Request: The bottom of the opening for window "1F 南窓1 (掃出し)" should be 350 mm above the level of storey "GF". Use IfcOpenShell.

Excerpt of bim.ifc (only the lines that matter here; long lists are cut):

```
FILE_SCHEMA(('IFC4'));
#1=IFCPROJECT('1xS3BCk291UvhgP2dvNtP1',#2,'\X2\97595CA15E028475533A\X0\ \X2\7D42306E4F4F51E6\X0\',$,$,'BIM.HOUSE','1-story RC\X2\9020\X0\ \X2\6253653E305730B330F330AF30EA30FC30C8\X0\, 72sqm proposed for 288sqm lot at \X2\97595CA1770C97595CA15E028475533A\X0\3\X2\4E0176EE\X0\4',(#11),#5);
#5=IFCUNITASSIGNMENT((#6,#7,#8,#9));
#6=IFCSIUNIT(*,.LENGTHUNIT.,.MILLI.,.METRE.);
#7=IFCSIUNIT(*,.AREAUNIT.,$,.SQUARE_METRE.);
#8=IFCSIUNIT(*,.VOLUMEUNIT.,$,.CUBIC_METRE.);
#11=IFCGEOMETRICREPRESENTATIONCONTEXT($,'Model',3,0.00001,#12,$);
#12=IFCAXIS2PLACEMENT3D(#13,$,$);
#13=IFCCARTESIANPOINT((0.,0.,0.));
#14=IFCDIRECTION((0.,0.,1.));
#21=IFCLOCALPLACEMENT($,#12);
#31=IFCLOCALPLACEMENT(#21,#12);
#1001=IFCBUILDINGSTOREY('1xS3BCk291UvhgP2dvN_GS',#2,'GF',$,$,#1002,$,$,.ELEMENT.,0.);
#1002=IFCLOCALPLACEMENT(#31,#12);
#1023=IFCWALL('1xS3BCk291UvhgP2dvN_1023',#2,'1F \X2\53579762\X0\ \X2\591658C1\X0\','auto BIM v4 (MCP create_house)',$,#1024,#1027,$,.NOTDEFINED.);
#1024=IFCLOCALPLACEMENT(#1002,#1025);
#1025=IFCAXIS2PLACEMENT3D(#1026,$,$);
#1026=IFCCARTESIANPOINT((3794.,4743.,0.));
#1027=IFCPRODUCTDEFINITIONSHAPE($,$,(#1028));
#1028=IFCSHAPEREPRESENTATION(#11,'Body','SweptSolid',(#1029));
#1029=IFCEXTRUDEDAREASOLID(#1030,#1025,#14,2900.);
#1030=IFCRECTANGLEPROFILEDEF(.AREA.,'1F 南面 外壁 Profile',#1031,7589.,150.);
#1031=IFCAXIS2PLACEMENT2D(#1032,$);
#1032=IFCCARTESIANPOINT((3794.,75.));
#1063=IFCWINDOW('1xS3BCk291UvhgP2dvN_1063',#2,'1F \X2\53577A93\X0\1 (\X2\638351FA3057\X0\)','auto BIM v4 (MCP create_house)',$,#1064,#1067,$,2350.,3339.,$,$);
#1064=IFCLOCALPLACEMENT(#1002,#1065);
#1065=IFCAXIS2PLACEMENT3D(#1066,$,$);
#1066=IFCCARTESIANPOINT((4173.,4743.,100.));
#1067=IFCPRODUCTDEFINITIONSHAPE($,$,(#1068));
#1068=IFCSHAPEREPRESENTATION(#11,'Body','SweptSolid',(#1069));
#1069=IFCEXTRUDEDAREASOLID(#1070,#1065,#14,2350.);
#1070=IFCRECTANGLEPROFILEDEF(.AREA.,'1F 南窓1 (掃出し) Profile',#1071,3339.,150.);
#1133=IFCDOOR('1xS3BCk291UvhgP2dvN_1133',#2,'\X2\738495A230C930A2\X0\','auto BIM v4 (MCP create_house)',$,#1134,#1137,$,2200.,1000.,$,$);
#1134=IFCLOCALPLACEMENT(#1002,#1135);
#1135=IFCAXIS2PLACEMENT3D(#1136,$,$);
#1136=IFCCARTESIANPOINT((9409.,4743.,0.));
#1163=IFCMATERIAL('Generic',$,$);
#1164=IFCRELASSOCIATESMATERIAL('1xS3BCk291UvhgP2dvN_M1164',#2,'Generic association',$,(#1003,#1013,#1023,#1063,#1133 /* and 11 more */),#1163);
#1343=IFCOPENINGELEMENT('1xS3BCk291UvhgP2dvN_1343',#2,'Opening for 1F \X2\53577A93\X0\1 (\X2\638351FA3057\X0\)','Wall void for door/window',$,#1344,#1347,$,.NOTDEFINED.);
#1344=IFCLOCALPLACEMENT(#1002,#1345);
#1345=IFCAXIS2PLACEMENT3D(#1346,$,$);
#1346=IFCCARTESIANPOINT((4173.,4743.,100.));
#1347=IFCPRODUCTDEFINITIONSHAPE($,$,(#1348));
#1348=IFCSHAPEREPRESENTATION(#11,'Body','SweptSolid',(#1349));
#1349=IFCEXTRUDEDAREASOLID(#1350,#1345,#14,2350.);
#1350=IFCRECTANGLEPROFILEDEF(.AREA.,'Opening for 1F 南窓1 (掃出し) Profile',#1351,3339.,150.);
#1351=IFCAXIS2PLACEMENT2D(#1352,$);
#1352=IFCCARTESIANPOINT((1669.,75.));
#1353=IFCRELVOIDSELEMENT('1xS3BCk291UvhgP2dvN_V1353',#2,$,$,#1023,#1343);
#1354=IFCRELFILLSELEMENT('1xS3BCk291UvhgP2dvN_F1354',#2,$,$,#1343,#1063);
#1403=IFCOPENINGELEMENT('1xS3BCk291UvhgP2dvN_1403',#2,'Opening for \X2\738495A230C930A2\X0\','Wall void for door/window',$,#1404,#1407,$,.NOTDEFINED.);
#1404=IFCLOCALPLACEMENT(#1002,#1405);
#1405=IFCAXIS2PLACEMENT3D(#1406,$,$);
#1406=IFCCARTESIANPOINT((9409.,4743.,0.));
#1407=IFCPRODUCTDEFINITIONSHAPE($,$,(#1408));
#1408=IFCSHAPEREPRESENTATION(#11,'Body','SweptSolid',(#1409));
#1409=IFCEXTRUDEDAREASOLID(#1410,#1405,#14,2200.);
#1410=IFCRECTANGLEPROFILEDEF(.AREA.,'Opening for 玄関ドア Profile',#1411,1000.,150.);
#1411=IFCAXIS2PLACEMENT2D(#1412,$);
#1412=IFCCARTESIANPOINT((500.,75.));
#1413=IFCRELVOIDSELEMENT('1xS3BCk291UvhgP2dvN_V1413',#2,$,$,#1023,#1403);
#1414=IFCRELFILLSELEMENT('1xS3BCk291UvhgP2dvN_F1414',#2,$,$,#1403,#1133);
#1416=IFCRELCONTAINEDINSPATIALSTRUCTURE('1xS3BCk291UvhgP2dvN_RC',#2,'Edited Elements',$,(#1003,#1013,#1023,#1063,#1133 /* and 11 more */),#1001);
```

```python
import numpy as np
import ifcopenshell
import ifcopenshell.api.geometry
import ifcopenshell.geom
import ifcopenshell.util.element
import ifcopenshell.util.placement
import ifcopenshell.util.shape
import ifcopenshell.util.unit

model = ifcopenshell.open("bim.ifc")
unit_scale = ifcopenshell.util.unit.calculate_unit_scale(model)

window = model.by_guid("1xS3BCk291UvhgP2dvN_1063")
opening = window.FillsVoids[0].RelatingOpeningElement
storey = ifcopenshell.util.element.get_container(window, ifc_class="IfcBuildingStorey")
level = ifcopenshell.util.placement.get_local_placement(storey.ObjectPlacement)[2, 3]

# The opening's origin need not be at the sill, so measure its lowest point.
shape = ifcopenshell.geom.create_shape(ifcopenshell.geom.settings(), opening)
bottom = ifcopenshell.util.shape.get_shape_bottom_elevation(shape, shape.geometry) / unit_scale
dz = level + 0.35 / unit_scale - bottom

shift = np.array([0.0, 0.0, dz])
# The window is not placed relative to its opening, so move both.
for product in (opening, window):
    matrix = ifcopenshell.util.placement.get_local_placement(product.ObjectPlacement)
    matrix[:3, 3] += shift
    ifcopenshell.api.geometry.edit_object_placement(model, product=product, matrix=matrix, is_si=False)

print(f"moved by {dz * unit_scale:+.3f} m")

model.write("bim_v2.ifc")
```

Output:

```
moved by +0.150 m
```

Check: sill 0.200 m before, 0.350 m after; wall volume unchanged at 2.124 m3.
